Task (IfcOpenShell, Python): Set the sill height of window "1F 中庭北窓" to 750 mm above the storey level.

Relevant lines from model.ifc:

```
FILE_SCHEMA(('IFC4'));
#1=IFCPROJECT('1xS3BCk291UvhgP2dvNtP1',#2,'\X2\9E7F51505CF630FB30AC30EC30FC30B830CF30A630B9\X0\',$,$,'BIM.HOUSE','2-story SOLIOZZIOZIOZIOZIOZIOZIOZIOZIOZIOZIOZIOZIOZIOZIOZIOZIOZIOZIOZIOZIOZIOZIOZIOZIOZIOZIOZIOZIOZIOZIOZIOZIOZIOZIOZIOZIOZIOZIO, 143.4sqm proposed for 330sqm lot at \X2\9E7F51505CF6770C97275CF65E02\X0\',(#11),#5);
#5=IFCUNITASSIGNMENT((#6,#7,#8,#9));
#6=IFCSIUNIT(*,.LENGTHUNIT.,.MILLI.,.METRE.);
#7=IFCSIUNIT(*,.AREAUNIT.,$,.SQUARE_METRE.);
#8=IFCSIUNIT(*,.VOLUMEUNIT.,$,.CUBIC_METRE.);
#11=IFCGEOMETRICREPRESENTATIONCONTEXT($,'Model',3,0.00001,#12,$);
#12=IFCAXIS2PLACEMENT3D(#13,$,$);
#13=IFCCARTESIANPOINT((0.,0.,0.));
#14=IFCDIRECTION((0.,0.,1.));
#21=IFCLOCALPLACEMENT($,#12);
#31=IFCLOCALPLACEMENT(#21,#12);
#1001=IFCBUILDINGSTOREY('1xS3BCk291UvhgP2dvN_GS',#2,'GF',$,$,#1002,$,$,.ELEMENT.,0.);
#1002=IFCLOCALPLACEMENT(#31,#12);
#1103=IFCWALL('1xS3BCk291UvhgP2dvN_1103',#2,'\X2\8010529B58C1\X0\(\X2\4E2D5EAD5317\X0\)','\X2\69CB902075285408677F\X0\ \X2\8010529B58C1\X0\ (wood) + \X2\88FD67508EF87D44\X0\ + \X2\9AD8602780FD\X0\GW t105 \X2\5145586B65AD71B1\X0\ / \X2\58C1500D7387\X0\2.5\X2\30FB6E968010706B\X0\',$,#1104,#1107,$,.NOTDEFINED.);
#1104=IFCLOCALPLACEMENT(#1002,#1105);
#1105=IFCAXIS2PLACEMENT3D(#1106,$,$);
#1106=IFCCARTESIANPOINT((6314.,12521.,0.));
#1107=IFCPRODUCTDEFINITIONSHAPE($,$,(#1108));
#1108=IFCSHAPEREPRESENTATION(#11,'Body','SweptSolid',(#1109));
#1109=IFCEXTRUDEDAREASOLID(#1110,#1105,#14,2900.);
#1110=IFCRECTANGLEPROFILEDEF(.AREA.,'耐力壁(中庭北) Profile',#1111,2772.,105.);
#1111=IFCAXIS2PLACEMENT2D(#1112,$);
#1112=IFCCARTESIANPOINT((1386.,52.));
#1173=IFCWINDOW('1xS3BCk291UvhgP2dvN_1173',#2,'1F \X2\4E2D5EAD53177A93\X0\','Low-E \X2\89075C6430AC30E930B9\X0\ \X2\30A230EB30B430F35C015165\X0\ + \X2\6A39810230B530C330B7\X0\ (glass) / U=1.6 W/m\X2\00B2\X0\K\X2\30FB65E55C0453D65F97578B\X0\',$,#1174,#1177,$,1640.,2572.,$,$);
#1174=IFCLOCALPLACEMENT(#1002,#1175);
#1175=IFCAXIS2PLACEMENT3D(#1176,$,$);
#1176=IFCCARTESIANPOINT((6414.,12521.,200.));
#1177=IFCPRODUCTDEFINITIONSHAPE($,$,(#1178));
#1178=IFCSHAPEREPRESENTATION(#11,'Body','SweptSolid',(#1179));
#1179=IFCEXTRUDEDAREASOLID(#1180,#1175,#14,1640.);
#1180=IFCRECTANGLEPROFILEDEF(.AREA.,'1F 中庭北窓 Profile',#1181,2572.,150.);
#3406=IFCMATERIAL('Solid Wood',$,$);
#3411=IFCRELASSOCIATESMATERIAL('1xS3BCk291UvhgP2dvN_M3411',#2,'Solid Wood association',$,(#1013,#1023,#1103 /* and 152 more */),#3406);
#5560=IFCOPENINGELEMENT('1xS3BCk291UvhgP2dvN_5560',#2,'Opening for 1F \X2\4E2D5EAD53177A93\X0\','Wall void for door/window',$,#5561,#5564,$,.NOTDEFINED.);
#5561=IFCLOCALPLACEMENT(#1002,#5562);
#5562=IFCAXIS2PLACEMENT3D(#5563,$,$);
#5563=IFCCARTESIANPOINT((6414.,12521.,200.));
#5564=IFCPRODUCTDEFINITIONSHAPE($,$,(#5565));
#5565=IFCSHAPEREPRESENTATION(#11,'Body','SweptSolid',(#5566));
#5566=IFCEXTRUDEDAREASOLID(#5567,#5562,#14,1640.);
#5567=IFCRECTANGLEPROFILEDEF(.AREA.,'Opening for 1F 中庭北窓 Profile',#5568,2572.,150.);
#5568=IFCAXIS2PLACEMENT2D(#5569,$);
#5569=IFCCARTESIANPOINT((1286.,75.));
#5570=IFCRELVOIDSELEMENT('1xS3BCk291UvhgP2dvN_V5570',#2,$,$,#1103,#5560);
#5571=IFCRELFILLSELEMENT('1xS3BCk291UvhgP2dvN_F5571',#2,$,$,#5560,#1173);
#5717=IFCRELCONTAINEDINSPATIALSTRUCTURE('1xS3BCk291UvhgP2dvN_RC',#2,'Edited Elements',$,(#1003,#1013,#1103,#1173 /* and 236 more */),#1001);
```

```python
import numpy as np
import ifcopenshell
import ifcopenshell.api.geometry
import ifcopenshell.geom
import ifcopenshell.util.element
import ifcopenshell.util.placement
import ifcopenshell.util.shape
import ifcopenshell.util.unit

model = ifcopenshell.open("model.ifc")
unit_scale = ifcopenshell.util.unit.calculate_unit_scale(model)

window = model.by_guid("1xS3BCk291UvhgP2dvN_1173")
opening = window.FillsVoids[0].RelatingOpeningElement
storey = ifcopenshell.util.element.get_container(window, ifc_class="IfcBuildingStorey")
level = ifcopenshell.util.placement.get_local_placement(storey.ObjectPlacement)[2, 3]

# The opening's origin need not be at the sill, so measure its lowest point.
shape = ifcopenshell.geom.create_shape(ifcopenshell.geom.settings(), opening)
bottom = ifcopenshell.util.shape.get_shape_bottom_elevation(shape, shape.geometry) / unit_scale
dz = level + 0.75 / unit_scale - bottom

shift = np.array([0.0, 0.0, dz])
# The window is not placed relative to its opening, so move both.
for product in (opening, window):
    matrix = ifcopenshell.util.placement.get_local_placement(product.ObjectPlacement)
    matrix[:3, 3] += shift
    ifcopenshell.api.geometry.edit_object_placement(model, product=product, matrix=matrix, is_si=False)

print(f"moved by {dz * unit_scale:+.3f} m")

model.write("model_rev.ifc")
```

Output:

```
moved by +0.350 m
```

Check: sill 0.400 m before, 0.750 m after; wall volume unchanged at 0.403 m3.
